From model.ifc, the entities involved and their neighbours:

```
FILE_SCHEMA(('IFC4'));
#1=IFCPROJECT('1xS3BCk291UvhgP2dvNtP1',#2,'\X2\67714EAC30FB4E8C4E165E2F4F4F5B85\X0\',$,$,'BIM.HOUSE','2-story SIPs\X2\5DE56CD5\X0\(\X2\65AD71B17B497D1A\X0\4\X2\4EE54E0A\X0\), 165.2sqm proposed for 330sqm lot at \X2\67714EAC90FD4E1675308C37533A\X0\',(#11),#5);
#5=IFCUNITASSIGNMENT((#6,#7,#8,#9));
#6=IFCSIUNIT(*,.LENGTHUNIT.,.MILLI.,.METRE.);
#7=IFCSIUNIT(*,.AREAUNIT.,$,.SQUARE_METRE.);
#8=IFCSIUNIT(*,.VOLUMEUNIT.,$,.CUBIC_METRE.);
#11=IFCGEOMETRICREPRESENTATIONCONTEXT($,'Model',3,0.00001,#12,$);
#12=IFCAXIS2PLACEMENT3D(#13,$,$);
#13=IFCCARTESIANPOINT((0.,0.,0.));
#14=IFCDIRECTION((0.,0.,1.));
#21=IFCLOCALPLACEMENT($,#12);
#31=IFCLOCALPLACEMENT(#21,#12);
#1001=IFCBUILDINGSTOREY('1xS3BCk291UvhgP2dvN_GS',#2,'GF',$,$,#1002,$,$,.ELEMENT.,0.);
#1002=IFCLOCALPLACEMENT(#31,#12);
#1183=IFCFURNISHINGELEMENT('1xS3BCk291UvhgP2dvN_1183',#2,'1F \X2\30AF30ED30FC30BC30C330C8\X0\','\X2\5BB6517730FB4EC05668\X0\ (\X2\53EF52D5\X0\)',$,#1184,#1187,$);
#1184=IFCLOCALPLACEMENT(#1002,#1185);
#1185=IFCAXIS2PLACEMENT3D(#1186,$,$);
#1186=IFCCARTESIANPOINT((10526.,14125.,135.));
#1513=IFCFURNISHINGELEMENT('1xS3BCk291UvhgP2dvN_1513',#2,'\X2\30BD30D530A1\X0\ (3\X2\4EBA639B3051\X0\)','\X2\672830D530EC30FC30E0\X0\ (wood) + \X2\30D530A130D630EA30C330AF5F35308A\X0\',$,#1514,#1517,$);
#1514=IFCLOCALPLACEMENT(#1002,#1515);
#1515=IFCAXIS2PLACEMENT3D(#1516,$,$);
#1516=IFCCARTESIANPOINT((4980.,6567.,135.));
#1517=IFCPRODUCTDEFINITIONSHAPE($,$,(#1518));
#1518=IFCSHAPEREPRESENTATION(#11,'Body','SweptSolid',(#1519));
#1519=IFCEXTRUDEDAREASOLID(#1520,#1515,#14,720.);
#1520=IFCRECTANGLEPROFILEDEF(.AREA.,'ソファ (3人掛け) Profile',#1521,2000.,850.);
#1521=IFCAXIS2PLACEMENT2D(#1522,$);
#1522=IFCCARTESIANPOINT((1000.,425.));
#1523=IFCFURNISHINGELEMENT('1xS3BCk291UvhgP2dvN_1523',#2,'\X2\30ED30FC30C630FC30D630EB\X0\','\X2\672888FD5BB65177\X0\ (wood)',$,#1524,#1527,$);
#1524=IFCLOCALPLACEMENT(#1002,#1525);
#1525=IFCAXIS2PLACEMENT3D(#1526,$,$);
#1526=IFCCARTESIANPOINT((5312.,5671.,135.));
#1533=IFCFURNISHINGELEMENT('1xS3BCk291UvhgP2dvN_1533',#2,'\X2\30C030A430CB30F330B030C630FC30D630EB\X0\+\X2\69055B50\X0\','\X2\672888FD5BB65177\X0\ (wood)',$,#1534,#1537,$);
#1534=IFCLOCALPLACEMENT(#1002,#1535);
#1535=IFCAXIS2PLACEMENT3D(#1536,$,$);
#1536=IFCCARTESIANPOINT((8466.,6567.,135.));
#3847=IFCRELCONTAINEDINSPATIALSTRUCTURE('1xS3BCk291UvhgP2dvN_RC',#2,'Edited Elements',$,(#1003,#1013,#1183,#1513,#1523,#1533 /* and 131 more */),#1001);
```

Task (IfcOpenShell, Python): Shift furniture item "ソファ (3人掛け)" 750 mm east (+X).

```python
import ifcopenshell
import ifcopenshell.api.geometry
import ifcopenshell.util.placement

model = ifcopenshell.open("model.ifc")

item = model.by_guid("1xS3BCk291UvhgP2dvN_1513")
matrix = ifcopenshell.util.placement.get_local_placement(item.ObjectPlacement)
matrix[0, 3] += 750.0
ifcopenshell.api.geometry.edit_object_placement(model, product=item, matrix=matrix, is_si=False)

print(ifcopenshell.util.placement.get_local_placement(item.ObjectPlacement).round(3) + 0.0)

model.write("model_v2.ifc")
```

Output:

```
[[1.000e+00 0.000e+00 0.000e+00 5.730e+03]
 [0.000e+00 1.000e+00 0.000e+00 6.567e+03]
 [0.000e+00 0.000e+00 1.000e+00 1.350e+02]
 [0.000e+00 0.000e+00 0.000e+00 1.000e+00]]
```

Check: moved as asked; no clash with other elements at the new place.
